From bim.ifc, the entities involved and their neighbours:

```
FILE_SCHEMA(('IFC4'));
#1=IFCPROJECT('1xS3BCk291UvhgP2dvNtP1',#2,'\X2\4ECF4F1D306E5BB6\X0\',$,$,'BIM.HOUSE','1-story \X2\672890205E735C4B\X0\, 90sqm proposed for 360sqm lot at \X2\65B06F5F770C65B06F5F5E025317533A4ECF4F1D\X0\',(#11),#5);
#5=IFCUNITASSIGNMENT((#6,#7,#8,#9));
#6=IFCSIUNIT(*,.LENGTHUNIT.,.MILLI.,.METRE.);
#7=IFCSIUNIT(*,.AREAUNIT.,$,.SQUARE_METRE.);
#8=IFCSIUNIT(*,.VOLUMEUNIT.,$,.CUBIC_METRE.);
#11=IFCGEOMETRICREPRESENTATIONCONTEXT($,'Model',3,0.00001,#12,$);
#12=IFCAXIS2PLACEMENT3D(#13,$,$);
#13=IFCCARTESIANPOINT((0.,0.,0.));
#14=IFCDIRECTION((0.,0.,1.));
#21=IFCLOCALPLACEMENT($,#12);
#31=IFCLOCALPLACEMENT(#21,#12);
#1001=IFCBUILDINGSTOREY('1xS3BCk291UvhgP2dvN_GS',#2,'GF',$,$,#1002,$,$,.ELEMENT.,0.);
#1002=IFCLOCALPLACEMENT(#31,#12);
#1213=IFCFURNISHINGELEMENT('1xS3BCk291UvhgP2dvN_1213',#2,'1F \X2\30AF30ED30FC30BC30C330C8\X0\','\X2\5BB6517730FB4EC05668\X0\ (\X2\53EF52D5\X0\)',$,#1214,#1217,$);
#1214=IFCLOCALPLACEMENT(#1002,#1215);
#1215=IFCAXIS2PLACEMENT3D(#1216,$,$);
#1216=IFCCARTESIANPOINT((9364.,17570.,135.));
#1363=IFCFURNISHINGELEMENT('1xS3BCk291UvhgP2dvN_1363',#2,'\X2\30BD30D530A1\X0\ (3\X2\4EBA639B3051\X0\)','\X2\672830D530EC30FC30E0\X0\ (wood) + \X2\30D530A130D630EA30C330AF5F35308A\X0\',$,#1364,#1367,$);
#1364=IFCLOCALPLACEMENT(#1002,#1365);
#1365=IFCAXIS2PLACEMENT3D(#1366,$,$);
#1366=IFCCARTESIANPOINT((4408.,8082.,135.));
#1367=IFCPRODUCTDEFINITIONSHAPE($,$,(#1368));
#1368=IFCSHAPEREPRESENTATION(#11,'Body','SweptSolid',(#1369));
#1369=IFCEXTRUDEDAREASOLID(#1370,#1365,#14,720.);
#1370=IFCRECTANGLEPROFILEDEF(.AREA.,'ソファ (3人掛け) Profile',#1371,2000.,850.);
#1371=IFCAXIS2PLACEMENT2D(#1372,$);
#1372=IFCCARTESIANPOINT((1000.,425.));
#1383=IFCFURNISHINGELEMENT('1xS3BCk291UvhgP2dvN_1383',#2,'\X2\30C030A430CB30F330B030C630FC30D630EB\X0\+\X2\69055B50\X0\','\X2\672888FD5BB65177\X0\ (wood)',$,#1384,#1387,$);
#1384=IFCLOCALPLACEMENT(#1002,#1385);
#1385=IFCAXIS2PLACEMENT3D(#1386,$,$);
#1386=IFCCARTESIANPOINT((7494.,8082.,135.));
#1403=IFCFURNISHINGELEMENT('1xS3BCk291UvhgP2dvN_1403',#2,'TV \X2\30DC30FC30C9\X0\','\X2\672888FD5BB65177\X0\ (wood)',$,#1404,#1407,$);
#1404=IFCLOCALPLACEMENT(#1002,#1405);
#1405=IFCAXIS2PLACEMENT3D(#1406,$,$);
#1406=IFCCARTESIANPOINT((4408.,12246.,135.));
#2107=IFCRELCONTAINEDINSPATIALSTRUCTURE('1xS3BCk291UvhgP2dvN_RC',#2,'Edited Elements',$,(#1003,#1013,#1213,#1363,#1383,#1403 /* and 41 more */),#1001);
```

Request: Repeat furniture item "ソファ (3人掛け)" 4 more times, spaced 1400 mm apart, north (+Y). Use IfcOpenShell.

```python
import numpy as np
import ifcopenshell
import ifcopenshell.api.geometry
import ifcopenshell.api.root
import ifcopenshell.util.element
import ifcopenshell.util.placement

model = ifcopenshell.open("bim.ifc")


def reuse_history(source, copy):
    """copy_class also copies each property set's owner history, people and application; keep the originals."""
    for rel in copy.IsDefinedBy:
        if rel.is_a("IfcRelDefinesByProperties") and (history := rel.RelatingPropertyDefinition.OwnerHistory):
            rel.RelatingPropertyDefinition.OwnerHistory = source.OwnerHistory
            ifcopenshell.util.element.remove_deep2(model, history)


source = model.by_id(1363)
base = ifcopenshell.util.placement.get_local_placement(source.ObjectPlacement)
step = np.array([0.0, 1.0, 0.0]) * 1400.0

for i in range(1, 5):
    copy = ifcopenshell.api.root.copy_class(model, product=source)
    copy.Representation = ifcopenshell.util.element.copy_deep(
        model, source.Representation, exclude=["IfcGeometricRepresentationContext", "IfcRepresentationMap"]
    )
    reuse_history(source, copy)
    matrix = base.copy()
    matrix[:3, 3] += i * step
    print("added at", matrix[:3, 3].round(3) + 0.0)
    ifcopenshell.api.geometry.edit_object_placement(model, product=copy, matrix=matrix, is_si=False)

model.write("bim_rev.ifc")
```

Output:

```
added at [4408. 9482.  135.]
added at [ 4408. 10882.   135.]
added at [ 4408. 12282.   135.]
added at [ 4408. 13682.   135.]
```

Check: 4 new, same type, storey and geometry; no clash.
